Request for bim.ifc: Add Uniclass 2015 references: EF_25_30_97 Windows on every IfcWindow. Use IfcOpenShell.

First a look at what the model holds.

```python
import ifcopenshell

model = ifcopenshell.open("bim.ifc")
print(model.schema)
print("classifications:", [c.Name for c in model.by_type("IfcClassification")])
for ifc_class in ("IfcDoor", "IfcRoof", "IfcStair", "IfcWall", "IfcWindow"):
    print(ifc_class, len(model.by_type(ifc_class)))
```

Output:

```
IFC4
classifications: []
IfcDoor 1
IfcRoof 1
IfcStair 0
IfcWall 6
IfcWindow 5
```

```python
import ifcopenshell
import ifcopenshell.api.classification

model = ifcopenshell.open("bim.ifc")

system = ifcopenshell.api.classification.add_classification(model, classification="Uniclass 2015")

codes = {
    "IfcWindow": ("EF_25_30_97", "Windows"),
}
for ifc_class, (code, name) in codes.items():
    products = model.by_type(ifc_class)
    ifcopenshell.api.classification.add_reference(
        model, products=products, classification=system, identification=code, name=name
    )
    print(code, len(products))

model.write("bim_updated.ifc")
```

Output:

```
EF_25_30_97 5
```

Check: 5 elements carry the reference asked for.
